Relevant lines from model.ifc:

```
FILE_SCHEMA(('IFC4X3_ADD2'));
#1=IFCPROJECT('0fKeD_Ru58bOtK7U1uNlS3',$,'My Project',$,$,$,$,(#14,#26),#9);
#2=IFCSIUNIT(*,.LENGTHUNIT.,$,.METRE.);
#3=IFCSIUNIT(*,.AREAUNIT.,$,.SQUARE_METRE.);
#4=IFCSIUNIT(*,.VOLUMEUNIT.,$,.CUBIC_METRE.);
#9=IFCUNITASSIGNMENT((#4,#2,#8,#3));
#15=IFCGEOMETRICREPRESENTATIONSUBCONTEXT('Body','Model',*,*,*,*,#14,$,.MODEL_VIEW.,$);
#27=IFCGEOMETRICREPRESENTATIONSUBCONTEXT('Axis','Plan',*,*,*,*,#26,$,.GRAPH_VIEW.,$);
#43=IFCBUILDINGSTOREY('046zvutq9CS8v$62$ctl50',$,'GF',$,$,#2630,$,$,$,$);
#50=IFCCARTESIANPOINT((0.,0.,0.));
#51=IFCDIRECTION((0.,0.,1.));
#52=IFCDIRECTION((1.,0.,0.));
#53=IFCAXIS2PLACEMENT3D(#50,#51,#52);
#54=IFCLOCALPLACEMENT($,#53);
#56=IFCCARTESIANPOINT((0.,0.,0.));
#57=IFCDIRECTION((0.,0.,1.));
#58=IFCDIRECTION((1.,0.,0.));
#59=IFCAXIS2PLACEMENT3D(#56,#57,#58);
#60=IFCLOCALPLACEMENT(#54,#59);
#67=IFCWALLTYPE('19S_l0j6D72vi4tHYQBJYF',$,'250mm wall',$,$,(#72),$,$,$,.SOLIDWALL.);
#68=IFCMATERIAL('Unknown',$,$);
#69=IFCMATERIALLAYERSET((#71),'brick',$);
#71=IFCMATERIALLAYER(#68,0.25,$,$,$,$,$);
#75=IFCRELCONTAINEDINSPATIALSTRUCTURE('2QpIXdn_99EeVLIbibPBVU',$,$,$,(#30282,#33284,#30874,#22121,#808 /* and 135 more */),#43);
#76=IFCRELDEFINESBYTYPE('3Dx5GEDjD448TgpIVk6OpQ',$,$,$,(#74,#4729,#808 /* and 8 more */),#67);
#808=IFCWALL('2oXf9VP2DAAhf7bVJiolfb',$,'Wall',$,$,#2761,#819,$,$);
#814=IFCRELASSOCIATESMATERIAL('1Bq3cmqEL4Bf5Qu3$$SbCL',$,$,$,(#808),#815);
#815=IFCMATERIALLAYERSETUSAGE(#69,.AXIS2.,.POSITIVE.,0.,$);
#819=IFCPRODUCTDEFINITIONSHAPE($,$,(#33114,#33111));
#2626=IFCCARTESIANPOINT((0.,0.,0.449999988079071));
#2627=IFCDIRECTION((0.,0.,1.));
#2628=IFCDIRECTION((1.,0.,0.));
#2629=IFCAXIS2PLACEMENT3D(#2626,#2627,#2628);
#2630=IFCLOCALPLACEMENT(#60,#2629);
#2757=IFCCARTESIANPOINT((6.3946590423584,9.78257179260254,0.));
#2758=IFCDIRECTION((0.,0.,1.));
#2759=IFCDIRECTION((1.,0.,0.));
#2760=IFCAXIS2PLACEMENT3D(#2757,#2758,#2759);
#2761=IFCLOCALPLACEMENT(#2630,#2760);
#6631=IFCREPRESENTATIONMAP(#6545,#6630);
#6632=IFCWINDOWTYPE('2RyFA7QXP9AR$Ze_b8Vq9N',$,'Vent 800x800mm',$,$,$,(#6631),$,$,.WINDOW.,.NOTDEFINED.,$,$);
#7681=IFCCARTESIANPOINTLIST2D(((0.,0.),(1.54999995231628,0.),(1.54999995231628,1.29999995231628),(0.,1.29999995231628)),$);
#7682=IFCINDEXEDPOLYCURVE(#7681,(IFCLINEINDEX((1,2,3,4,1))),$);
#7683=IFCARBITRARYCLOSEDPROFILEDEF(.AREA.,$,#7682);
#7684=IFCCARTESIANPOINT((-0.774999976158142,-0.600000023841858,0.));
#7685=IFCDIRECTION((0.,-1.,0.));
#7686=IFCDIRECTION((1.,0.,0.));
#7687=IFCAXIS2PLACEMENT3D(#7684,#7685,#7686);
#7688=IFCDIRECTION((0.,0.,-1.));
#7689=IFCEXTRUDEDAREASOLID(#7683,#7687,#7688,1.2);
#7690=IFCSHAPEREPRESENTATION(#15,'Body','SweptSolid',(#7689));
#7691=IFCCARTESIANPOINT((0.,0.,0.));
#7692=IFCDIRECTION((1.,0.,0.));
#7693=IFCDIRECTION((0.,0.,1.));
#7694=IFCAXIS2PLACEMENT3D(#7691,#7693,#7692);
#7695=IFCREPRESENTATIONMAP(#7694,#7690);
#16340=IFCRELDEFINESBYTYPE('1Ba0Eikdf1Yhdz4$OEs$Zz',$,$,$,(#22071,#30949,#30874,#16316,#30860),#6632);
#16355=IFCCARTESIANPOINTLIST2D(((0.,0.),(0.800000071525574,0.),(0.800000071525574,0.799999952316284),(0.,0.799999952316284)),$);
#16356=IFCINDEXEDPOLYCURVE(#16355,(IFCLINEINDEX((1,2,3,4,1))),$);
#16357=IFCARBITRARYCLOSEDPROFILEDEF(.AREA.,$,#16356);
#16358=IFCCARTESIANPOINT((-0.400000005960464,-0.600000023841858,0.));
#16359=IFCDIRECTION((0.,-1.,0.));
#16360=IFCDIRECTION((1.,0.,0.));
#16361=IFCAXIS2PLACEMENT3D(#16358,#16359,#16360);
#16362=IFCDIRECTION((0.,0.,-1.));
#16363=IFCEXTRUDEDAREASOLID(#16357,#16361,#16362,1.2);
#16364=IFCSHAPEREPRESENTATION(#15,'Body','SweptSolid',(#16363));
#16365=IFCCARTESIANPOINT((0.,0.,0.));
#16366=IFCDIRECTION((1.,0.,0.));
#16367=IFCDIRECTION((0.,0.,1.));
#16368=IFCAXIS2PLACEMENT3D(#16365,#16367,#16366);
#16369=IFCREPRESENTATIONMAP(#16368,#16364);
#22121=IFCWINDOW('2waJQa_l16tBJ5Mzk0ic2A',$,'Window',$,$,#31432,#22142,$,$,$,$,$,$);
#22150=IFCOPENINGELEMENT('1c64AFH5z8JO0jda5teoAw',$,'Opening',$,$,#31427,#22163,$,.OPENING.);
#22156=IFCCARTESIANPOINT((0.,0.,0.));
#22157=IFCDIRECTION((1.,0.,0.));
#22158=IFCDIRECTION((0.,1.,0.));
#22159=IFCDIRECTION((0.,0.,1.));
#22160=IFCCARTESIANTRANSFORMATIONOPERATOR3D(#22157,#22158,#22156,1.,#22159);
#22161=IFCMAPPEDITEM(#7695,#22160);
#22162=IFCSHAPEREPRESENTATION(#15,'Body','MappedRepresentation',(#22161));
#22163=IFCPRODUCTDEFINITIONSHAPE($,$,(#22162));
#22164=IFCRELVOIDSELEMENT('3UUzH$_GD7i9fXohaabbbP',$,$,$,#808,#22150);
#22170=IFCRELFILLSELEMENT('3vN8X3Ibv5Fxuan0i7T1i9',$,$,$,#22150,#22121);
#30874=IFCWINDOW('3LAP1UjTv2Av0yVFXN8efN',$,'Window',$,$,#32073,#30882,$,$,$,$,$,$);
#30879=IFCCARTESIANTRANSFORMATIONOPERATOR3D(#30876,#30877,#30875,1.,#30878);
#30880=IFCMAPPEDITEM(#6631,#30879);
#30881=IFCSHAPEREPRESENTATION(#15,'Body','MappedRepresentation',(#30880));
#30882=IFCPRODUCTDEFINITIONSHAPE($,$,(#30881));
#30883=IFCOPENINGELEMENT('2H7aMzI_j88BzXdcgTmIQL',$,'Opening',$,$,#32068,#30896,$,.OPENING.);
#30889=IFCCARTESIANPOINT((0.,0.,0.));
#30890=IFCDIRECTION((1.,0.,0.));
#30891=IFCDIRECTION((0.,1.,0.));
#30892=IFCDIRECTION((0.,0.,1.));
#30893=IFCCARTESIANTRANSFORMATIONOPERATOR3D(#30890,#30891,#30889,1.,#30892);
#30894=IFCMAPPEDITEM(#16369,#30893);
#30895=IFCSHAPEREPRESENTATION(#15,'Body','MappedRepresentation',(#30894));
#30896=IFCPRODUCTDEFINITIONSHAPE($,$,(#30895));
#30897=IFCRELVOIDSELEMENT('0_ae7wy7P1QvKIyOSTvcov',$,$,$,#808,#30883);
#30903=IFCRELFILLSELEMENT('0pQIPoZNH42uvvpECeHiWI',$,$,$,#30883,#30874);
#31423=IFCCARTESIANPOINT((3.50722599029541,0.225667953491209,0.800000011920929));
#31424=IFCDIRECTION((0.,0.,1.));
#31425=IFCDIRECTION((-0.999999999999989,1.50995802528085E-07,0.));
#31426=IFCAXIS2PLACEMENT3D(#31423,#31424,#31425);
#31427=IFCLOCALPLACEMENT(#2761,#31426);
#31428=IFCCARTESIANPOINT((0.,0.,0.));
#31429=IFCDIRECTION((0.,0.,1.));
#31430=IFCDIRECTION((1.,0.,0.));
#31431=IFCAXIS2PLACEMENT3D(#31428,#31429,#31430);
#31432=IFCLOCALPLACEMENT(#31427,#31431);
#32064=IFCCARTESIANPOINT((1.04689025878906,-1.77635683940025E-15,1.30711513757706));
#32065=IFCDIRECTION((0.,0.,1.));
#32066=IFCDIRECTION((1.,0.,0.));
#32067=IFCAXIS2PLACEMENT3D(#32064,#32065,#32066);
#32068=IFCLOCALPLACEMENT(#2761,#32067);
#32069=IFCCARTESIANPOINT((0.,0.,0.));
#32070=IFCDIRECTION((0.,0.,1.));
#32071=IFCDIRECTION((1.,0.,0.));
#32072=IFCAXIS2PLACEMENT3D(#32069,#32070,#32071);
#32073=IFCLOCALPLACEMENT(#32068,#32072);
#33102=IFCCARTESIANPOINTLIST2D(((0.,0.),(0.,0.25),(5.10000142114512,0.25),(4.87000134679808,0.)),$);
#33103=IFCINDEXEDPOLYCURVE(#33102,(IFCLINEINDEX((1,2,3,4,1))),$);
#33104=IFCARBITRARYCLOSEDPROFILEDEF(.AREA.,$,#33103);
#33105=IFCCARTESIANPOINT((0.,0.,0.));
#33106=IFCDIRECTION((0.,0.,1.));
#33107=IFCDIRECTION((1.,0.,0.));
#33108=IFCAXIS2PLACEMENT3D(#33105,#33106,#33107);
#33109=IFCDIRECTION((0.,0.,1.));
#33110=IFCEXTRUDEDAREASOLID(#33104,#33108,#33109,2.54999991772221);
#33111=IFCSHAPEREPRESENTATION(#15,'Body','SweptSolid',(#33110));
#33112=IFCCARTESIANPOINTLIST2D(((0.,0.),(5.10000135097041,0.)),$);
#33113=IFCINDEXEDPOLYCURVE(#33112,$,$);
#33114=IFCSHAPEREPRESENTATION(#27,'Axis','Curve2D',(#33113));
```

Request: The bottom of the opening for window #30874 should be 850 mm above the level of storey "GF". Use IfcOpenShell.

```python
import numpy as np
import ifcopenshell
import ifcopenshell.api.geometry
import ifcopenshell.geom
import ifcopenshell.util.element
import ifcopenshell.util.placement
import ifcopenshell.util.shape
import ifcopenshell.util.unit

model = ifcopenshell.open("model.ifc")
unit_scale = ifcopenshell.util.unit.calculate_unit_scale(model)

window = model.by_guid("3LAP1UjTv2Av0yVFXN8efN")
opening = window.FillsVoids[0].RelatingOpeningElement
storey = ifcopenshell.util.element.get_container(window, ifc_class="IfcBuildingStorey")
level = ifcopenshell.util.placement.get_local_placement(storey.ObjectPlacement)[2, 3]

# The opening's origin need not be at the sill, so measure its lowest point.
shape = ifcopenshell.geom.create_shape(ifcopenshell.geom.settings(), opening)
bottom = ifcopenshell.util.shape.get_shape_bottom_elevation(shape, shape.geometry) / unit_scale
dz = level + 0.85 - bottom

shift = np.array([0.0, 0.0, dz])
# The window is placed relative to its opening, so it follows when the opening moves.
matrix = ifcopenshell.util.placement.get_local_placement(opening.ObjectPlacement)
matrix[:3, 3] += shift
ifcopenshell.api.geometry.edit_object_placement(
    model, product=opening, matrix=matrix, is_si=False, should_transform_children=True
)

print(f"moved by {dz * unit_scale:+.3f} m")

model.write("model_updated.ifc")
```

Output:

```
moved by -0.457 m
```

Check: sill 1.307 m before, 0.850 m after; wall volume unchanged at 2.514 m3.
